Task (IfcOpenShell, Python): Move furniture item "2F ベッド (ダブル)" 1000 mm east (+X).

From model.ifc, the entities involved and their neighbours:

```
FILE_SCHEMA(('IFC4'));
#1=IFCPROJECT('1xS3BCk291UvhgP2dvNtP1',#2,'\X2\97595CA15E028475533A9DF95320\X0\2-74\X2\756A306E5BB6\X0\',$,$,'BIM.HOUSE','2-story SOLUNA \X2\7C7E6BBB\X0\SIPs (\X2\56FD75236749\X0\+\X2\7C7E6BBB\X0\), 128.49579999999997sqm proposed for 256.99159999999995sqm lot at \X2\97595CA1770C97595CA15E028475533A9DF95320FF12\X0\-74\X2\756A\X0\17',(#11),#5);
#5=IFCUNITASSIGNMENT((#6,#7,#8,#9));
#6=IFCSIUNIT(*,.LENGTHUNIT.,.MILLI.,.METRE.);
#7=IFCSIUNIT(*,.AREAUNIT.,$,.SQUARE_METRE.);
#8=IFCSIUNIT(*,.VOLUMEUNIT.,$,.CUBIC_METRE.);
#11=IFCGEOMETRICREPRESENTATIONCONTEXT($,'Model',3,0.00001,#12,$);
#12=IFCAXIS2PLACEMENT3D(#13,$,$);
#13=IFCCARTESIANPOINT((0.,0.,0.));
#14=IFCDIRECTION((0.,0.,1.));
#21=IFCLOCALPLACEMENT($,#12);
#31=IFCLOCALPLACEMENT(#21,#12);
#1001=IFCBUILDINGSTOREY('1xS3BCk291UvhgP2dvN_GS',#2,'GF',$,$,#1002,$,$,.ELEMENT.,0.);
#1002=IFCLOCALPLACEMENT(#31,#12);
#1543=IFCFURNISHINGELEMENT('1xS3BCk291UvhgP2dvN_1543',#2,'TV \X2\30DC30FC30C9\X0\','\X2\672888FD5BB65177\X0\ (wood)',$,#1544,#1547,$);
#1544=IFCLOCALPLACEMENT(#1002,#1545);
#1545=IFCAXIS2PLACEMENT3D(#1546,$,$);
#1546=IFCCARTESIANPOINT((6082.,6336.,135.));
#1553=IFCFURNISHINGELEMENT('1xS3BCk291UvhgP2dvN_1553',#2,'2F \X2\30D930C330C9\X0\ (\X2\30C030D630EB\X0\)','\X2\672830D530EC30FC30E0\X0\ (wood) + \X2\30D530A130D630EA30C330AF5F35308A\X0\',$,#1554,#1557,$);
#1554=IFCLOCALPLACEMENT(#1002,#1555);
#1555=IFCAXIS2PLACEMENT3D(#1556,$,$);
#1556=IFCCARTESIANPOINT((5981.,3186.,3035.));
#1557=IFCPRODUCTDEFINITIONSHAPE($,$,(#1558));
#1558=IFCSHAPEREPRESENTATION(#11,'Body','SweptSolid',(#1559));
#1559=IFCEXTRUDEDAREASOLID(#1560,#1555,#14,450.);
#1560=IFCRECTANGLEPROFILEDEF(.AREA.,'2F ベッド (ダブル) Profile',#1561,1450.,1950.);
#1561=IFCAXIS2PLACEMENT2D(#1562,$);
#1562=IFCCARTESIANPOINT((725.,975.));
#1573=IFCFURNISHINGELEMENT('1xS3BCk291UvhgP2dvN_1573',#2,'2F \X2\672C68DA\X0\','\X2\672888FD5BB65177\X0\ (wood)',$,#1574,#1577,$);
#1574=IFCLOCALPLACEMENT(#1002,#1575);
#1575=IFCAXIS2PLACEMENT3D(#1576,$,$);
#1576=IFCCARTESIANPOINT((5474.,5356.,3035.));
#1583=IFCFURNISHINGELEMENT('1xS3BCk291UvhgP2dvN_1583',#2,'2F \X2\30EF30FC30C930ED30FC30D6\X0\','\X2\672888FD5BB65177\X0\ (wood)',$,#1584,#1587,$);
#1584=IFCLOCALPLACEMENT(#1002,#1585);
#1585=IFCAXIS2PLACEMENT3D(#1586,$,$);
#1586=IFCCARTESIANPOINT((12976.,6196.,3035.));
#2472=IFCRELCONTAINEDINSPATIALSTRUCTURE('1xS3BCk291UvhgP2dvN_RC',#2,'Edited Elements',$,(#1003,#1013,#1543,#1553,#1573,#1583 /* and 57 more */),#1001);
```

```python
import ifcopenshell
import ifcopenshell.api.geometry
import ifcopenshell.util.placement
import ifcopenshell.util.unit

model = ifcopenshell.open("model.ifc")
unit_scale = ifcopenshell.util.unit.calculate_unit_scale(model)

item = model.by_guid("1xS3BCk291UvhgP2dvN_1553")
matrix = ifcopenshell.util.placement.get_local_placement(item.ObjectPlacement)
matrix[0, 3] += 1 / unit_scale
ifcopenshell.api.geometry.edit_object_placement(model, product=item, matrix=matrix, is_si=False)

print(ifcopenshell.util.placement.get_local_placement(item.ObjectPlacement).round(3) + 0.0)

model.write("model_updated.ifc")
```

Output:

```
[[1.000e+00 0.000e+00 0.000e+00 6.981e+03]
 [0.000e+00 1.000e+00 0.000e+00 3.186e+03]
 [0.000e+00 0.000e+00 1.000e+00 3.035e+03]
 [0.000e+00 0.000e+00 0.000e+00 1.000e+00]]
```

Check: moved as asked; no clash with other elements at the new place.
